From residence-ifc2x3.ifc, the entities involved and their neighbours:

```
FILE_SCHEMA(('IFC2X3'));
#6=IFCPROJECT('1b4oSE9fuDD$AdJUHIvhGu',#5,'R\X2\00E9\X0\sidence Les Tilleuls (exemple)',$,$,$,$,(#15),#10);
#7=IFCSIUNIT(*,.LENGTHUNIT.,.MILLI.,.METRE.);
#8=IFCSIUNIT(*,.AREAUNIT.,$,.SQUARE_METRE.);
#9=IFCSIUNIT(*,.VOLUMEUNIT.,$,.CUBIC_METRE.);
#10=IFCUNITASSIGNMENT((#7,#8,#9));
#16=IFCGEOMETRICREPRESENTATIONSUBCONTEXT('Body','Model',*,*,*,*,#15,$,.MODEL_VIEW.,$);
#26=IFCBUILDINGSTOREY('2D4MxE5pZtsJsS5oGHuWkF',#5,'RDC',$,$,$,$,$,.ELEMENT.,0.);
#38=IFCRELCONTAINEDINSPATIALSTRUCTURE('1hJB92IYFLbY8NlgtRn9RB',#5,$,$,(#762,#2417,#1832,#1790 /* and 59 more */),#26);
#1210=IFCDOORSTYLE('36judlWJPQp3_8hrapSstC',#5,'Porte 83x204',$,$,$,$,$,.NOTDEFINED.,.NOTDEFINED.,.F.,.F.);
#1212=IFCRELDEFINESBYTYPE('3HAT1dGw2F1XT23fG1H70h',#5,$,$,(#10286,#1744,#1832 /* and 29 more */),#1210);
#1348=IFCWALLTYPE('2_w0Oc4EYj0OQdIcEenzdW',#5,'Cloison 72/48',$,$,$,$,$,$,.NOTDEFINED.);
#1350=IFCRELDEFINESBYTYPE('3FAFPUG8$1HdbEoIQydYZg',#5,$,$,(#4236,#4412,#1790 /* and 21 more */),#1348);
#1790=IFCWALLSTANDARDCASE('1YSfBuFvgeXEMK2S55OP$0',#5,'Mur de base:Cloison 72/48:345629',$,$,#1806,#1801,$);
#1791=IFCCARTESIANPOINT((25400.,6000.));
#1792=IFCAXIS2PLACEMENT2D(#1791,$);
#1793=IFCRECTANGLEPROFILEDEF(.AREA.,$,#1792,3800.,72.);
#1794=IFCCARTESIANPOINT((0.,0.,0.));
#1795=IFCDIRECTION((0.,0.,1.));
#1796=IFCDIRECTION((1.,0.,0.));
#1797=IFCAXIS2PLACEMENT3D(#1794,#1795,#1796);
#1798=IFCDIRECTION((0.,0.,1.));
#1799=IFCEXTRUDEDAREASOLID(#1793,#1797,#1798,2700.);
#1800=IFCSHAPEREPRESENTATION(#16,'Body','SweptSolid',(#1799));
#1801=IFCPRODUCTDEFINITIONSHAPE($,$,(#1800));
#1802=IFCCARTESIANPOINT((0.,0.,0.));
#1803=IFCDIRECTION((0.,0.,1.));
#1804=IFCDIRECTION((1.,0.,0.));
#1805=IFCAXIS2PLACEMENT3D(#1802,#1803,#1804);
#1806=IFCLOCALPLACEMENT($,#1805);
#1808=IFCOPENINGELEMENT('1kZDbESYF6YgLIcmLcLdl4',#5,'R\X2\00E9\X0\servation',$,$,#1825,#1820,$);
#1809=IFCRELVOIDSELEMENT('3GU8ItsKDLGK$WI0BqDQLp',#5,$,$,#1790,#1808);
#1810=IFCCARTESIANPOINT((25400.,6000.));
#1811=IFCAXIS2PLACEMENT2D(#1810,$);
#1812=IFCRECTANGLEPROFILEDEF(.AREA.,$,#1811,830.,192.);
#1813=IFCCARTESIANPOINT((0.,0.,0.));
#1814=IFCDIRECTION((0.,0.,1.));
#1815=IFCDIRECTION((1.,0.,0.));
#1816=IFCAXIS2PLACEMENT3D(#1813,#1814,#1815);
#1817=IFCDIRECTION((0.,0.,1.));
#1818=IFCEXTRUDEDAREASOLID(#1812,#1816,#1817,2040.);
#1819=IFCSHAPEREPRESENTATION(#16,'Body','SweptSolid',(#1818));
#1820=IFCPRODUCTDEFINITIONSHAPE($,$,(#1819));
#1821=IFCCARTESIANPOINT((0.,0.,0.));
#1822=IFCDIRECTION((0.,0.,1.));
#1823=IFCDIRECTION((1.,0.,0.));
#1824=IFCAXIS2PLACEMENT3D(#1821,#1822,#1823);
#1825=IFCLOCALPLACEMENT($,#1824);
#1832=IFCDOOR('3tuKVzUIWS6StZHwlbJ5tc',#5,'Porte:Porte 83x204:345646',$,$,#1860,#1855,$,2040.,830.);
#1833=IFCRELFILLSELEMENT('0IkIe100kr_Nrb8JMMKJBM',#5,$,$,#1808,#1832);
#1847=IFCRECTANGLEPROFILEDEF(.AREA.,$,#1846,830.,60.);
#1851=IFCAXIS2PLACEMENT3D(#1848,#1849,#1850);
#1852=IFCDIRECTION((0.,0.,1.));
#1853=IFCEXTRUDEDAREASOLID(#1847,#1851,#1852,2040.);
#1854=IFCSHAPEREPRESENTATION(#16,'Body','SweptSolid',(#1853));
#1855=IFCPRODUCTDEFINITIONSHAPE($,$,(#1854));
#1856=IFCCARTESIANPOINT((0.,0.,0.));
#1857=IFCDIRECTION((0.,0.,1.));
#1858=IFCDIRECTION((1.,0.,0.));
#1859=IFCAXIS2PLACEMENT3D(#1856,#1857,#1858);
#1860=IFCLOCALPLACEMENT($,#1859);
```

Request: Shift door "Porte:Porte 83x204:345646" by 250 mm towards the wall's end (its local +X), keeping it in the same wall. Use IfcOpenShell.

```python
import ifcopenshell
import ifcopenshell.api.geometry
import ifcopenshell.util.placement
import ifcopenshell.util.unit

model = ifcopenshell.open("residence-ifc2x3.ifc")
unit_scale = ifcopenshell.util.unit.calculate_unit_scale(model)

door = model.by_guid("3tuKVzUIWS6StZHwlbJ5tc")
opening = door.FillsVoids[0].RelatingOpeningElement
wall = opening.VoidsElements[0].RelatingBuildingElement

wall_matrix = ifcopenshell.util.placement.get_local_placement(wall.ObjectPlacement)
shift = wall_matrix[:3, 0] * 0.25 / unit_scale
before = ifcopenshell.util.placement.get_local_placement(door.ObjectPlacement)[:3, 3].copy()

# The door is not placed relative to its opening, so move both.
for product in (opening, door):
    matrix = ifcopenshell.util.placement.get_local_placement(product.ObjectPlacement)
    matrix[:3, 3] += shift
    ifcopenshell.api.geometry.edit_object_placement(model, product=product, matrix=matrix, is_si=False)

after = ifcopenshell.util.placement.get_local_placement(door.ObjectPlacement)[:3, 3]
print("door moved by", (after - before).round(3) + 0.0)

model.write("residence-ifc2x3_rev.ifc")
```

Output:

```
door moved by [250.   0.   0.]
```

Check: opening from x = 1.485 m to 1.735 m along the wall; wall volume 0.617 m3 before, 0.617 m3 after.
